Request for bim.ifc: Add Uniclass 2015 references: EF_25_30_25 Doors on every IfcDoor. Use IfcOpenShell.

First a look at what the model holds.

```python
import ifcopenshell

model = ifcopenshell.open("bim.ifc")
print(model.schema)
print("classifications:", [c.Name for c in model.by_type("IfcClassification")])
for ifc_class in ("IfcDoor", "IfcRoof", "IfcStair", "IfcWall", "IfcWindow"):
    print(ifc_class, len(model.by_type(ifc_class)))
```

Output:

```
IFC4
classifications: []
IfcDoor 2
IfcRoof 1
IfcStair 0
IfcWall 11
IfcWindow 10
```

```python
import ifcopenshell
import ifcopenshell.api.classification

model = ifcopenshell.open("bim.ifc")

system = ifcopenshell.api.classification.add_classification(model, classification="Uniclass 2015")

codes = {
    "IfcDoor": ("EF_25_30_25", "Doors"),
}
for ifc_class, (code, name) in codes.items():
    products = model.by_type(ifc_class)
    ifcopenshell.api.classification.add_reference(
        model, products=products, classification=system, identification=code, name=name
    )
    print(code, len(products))

model.write("bim_edited.ifc")
```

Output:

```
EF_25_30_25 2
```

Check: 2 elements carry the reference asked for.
